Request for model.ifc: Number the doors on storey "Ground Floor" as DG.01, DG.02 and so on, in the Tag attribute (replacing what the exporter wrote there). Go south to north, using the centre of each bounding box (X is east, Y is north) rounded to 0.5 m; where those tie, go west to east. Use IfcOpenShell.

First a look at what the model holds.

```python
import ifcopenshell
import ifcopenshell.util.element
import ifcopenshell.util.placement

model = ifcopenshell.open("model.ifc")
print(model.schema)
storey = next(s for s in model.by_type("IfcBuildingStorey") if s.Name == "Ground Floor")
doors = [e for e in ifcopenshell.util.element.get_decomposition(storey) if e.is_a("IfcDoor")]
for e in sorted(doors, key=lambda e: e.id()):
    origin = ifcopenshell.util.placement.get_local_placement(e.ObjectPlacement)[:3, 3]
    print(e.id(), e.Tag, e.Name, origin.round(2) + 0.0, sep=" | ")
```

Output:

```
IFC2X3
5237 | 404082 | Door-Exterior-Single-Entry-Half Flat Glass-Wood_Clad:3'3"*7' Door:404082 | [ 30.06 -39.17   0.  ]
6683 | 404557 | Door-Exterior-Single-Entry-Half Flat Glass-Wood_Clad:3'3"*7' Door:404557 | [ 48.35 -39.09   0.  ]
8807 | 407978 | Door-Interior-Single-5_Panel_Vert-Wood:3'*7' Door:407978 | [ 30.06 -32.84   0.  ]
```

```python
import ifcopenshell
import ifcopenshell.geom
import ifcopenshell.util.element
import ifcopenshell.util.shape

model = ifcopenshell.open("model.ifc")
settings = ifcopenshell.geom.settings()
settings.set("use-world-coords", True)


def centre(element):
    shape = ifcopenshell.geom.create_shape(settings, element)
    return ifcopenshell.util.shape.get_bbox_centroid(shape.geometry)


storey = next(s for s in model.by_type("IfcBuildingStorey") if s.Name == "Ground Floor")
doors = [e for e in ifcopenshell.util.element.get_decomposition(storey) if e.is_a("IfcDoor")]

# Insertion points can sit at a corner or the storey origin, so sort by the geometry (in metres).
centres = {e: centre(e) for e in doors}
doors.sort(key=lambda e: (round(centres[e][1] / 0.5), centres[e][0]))

for i, e in enumerate(doors, start=1):
    number = f"DG.{i:02d}"
    e.Tag = number
    print(e.id(), number)

model.write("model_rev.ifc")
```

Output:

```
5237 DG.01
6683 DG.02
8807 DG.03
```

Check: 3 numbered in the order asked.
